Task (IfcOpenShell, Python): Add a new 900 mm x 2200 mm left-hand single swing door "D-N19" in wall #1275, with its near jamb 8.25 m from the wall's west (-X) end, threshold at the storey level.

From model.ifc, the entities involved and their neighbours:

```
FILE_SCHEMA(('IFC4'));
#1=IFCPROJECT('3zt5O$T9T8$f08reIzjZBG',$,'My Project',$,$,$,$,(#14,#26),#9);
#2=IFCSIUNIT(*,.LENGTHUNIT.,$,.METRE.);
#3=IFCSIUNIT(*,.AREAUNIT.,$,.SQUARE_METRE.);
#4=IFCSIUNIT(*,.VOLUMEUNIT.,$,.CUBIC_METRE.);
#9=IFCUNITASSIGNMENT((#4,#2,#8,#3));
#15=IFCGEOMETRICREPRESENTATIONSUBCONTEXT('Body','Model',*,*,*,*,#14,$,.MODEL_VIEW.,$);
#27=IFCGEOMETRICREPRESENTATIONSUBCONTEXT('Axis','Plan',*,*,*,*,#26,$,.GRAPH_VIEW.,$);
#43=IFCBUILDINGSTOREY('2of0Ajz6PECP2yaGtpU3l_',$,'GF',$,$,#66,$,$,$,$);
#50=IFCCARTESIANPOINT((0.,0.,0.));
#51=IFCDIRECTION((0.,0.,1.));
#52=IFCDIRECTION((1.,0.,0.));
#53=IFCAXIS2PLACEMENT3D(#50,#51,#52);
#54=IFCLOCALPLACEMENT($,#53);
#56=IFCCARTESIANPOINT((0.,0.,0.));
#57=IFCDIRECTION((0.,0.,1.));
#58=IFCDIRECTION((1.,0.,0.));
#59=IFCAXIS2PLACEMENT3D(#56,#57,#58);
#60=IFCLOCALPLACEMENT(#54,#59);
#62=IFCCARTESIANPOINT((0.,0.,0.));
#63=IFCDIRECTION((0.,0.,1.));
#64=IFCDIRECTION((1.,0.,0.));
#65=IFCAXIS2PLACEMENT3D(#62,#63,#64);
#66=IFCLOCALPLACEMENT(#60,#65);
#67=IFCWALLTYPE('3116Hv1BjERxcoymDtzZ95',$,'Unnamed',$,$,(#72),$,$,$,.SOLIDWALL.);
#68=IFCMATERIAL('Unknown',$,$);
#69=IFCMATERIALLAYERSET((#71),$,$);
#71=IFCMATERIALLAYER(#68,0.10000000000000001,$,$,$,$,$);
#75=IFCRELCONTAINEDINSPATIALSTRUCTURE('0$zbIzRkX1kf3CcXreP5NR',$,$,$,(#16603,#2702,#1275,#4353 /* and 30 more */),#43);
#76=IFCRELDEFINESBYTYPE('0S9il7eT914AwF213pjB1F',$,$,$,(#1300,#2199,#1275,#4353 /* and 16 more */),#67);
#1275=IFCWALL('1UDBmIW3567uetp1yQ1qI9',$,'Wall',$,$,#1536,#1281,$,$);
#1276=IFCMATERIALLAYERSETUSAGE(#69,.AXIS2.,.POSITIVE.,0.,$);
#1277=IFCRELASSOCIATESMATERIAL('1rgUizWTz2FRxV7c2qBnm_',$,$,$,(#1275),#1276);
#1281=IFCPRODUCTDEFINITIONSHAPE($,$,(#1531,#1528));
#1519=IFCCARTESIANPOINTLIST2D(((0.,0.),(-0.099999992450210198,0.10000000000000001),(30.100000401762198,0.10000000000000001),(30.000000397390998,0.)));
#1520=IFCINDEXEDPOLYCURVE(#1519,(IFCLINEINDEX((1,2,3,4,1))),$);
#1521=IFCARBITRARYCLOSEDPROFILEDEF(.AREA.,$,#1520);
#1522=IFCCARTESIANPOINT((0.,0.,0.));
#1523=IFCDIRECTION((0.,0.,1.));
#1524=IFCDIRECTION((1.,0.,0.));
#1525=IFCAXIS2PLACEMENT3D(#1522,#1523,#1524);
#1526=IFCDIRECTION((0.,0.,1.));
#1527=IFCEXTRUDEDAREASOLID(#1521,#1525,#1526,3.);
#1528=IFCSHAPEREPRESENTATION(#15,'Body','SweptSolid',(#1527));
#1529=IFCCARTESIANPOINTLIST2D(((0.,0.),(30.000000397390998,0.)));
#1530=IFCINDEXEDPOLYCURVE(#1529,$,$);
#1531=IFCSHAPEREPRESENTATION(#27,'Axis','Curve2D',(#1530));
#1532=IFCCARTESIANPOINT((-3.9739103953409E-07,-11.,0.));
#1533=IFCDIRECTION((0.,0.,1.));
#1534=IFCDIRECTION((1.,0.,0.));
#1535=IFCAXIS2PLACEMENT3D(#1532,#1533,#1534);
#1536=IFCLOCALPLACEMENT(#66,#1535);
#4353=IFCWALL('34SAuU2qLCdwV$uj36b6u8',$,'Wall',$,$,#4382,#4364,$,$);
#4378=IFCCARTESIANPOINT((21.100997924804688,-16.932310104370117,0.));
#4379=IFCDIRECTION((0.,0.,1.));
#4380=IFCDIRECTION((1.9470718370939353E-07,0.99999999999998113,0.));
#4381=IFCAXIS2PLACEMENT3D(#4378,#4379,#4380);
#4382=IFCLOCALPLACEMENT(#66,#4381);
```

```python
import numpy as np
import ifcopenshell
import ifcopenshell.api.feature
import ifcopenshell.api.geometry
import ifcopenshell.api.root
import ifcopenshell.api.spatial
import ifcopenshell.geom
import ifcopenshell.util.element
import ifcopenshell.util.placement
import ifcopenshell.util.representation
import ifcopenshell.util.shape
import ifcopenshell.util.unit

model = ifcopenshell.open("model.ifc")
unit_scale = ifcopenshell.util.unit.calculate_unit_scale(model)
settings = ifcopenshell.geom.settings()


def volume(element):
    """Net volume in cubic metres, openings subtracted."""
    shape = ifcopenshell.geom.create_shape(settings, element)
    return ifcopenshell.util.shape.get_volume(shape.geometry)


wall = model.by_guid("1UDBmIW3567uetp1yQ1qI9")
storey = ifcopenshell.util.element.get_container(wall, ifc_class="IfcBuildingStorey")
context = ifcopenshell.util.representation.get_context(model, "Model", "Body", "MODEL_VIEW")
before = volume(wall)

width, height, from_end, sill = 0.9, 2.2, 8.25, 0.0  # metres

# The wall runs along its own X axis, and the end named is its -X end.
wall_shape = ifcopenshell.geom.create_shape(settings, wall)
x, y, z = ifcopenshell.util.shape.get_vertices(wall_shape.geometry).T
start = x.min() + from_end
face, thickness = float(y.min()), float(y.max() - y.min())
wall_matrix = ifcopenshell.util.placement.get_local_placement(wall.ObjectPlacement)
level = ifcopenshell.util.placement.get_local_placement(storey.ObjectPlacement)[2, 3]


def in_wall(x, y):
    """Placement at x, y metres in the wall's axes, at sill height."""
    matrix = wall_matrix.copy()
    matrix[:, 3] = wall_matrix @ np.array([x / unit_scale, y / unit_scale, 0.0, 1.0])
    matrix[2, 3] = level + sill / unit_scale
    return matrix


# Opening: a box that overshoots both wall faces by 50 mm.
opening = ifcopenshell.api.root.create_entity(model, ifc_class="IfcOpeningElement", predefined_type="OPENING")
box = ifcopenshell.api.geometry.add_wall_representation(
    model, context=context, length=width, height=height, thickness=thickness + 0.1
)
ifcopenshell.api.geometry.assign_representation(model, product=opening, representation=box)
ifcopenshell.api.geometry.edit_object_placement(model, product=opening, matrix=in_wall(start, face - 0.05), is_si=False)
ifcopenshell.api.feature.add_feature(model, feature=opening, element=wall)

door = ifcopenshell.api.root.create_entity(model, ifc_class="IfcDoor", name="D-N19", predefined_type="DOOR")
door.OverallWidth, door.OverallHeight = width / unit_scale, height / unit_scale
door.OperationType = "SINGLE_SWING_LEFT"
body = ifcopenshell.api.geometry.add_door_representation(
    model,
    context=context,
    overall_width=door.OverallWidth,
    overall_height=door.OverallHeight,
    operation_type="SINGLE_SWING_LEFT",
    lining_properties={"LiningDepth": thickness / unit_scale, "ThresholdDepth": thickness / unit_scale},
)
ifcopenshell.api.geometry.assign_representation(model, product=door, representation=body)
ifcopenshell.api.spatial.assign_container(model, products=[door], relating_structure=storey)
ifcopenshell.api.feature.add_filling(model, opening=opening, element=door)

# The lining spans the wall, so the door starts at the wall face.
ifcopenshell.api.geometry.edit_object_placement(model, product=door, matrix=in_wall(start, face), is_si=False)

after = volume(wall)

print(f"wall volume {before:.3f} -> {after:.3f} m3")

model.write("model_updated.ifc")
```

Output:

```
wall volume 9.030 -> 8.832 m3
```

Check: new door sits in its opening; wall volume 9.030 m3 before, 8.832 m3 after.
